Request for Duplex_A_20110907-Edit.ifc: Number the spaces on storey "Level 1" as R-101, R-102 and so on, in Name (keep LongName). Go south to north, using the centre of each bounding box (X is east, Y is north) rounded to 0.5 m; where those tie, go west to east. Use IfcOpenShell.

First a look at what the model holds.

```python
import ifcopenshell
import ifcopenshell.util.element
import ifcopenshell.util.placement

model = ifcopenshell.open("Duplex_A_20110907-Edit.ifc")
print(model.schema)
storey = next(s for s in model.by_type("IfcBuildingStorey") if s.Name == "Level 1")
spaces = [e for e in ifcopenshell.util.element.get_decomposition(storey) if e.is_a("IfcSpace")]
for e in sorted(spaces, key=lambda e: e.id()):
    origin = ifcopenshell.util.placement.get_local_placement(e.ObjectPlacement)[:3, 3]
    print(e.id(), e.Name, e.LongName, origin.round(2) + 0.0, sep=" | ")
```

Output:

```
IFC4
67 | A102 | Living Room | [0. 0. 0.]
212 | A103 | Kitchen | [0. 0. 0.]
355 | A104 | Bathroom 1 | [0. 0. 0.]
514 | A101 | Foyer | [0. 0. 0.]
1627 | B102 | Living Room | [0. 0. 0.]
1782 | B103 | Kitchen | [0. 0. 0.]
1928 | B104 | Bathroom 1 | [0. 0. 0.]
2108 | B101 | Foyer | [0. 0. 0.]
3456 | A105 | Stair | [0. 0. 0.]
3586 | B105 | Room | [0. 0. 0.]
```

```python
import ifcopenshell
import ifcopenshell.geom
import ifcopenshell.util.element
import ifcopenshell.util.shape

model = ifcopenshell.open("Duplex_A_20110907-Edit.ifc")
settings = ifcopenshell.geom.settings()
settings.set("use-world-coords", True)


def centre(element):
    shape = ifcopenshell.geom.create_shape(settings, element)
    return ifcopenshell.util.shape.get_bbox_centroid(shape.geometry)


storey = next(s for s in model.by_type("IfcBuildingStorey") if s.Name == "Level 1")
spaces = [e for e in ifcopenshell.util.element.get_decomposition(storey) if e.is_a("IfcSpace")]

# Insertion points can sit at a corner or the storey origin, so sort by the geometry (in metres).
centres = {e: centre(e) for e in spaces}
spaces.sort(key=lambda e: (round(centres[e][1] / 0.5), centres[e][0]))

for i, e in enumerate(spaces, start=1):
    number = f"R-1{i:02d}"
    e.Name = number
    print(e.id(), number)

model.write("Duplex_A_20110907-Edit_rev.ifc")
```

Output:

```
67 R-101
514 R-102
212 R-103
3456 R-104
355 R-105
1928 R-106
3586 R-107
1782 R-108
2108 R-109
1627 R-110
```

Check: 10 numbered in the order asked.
